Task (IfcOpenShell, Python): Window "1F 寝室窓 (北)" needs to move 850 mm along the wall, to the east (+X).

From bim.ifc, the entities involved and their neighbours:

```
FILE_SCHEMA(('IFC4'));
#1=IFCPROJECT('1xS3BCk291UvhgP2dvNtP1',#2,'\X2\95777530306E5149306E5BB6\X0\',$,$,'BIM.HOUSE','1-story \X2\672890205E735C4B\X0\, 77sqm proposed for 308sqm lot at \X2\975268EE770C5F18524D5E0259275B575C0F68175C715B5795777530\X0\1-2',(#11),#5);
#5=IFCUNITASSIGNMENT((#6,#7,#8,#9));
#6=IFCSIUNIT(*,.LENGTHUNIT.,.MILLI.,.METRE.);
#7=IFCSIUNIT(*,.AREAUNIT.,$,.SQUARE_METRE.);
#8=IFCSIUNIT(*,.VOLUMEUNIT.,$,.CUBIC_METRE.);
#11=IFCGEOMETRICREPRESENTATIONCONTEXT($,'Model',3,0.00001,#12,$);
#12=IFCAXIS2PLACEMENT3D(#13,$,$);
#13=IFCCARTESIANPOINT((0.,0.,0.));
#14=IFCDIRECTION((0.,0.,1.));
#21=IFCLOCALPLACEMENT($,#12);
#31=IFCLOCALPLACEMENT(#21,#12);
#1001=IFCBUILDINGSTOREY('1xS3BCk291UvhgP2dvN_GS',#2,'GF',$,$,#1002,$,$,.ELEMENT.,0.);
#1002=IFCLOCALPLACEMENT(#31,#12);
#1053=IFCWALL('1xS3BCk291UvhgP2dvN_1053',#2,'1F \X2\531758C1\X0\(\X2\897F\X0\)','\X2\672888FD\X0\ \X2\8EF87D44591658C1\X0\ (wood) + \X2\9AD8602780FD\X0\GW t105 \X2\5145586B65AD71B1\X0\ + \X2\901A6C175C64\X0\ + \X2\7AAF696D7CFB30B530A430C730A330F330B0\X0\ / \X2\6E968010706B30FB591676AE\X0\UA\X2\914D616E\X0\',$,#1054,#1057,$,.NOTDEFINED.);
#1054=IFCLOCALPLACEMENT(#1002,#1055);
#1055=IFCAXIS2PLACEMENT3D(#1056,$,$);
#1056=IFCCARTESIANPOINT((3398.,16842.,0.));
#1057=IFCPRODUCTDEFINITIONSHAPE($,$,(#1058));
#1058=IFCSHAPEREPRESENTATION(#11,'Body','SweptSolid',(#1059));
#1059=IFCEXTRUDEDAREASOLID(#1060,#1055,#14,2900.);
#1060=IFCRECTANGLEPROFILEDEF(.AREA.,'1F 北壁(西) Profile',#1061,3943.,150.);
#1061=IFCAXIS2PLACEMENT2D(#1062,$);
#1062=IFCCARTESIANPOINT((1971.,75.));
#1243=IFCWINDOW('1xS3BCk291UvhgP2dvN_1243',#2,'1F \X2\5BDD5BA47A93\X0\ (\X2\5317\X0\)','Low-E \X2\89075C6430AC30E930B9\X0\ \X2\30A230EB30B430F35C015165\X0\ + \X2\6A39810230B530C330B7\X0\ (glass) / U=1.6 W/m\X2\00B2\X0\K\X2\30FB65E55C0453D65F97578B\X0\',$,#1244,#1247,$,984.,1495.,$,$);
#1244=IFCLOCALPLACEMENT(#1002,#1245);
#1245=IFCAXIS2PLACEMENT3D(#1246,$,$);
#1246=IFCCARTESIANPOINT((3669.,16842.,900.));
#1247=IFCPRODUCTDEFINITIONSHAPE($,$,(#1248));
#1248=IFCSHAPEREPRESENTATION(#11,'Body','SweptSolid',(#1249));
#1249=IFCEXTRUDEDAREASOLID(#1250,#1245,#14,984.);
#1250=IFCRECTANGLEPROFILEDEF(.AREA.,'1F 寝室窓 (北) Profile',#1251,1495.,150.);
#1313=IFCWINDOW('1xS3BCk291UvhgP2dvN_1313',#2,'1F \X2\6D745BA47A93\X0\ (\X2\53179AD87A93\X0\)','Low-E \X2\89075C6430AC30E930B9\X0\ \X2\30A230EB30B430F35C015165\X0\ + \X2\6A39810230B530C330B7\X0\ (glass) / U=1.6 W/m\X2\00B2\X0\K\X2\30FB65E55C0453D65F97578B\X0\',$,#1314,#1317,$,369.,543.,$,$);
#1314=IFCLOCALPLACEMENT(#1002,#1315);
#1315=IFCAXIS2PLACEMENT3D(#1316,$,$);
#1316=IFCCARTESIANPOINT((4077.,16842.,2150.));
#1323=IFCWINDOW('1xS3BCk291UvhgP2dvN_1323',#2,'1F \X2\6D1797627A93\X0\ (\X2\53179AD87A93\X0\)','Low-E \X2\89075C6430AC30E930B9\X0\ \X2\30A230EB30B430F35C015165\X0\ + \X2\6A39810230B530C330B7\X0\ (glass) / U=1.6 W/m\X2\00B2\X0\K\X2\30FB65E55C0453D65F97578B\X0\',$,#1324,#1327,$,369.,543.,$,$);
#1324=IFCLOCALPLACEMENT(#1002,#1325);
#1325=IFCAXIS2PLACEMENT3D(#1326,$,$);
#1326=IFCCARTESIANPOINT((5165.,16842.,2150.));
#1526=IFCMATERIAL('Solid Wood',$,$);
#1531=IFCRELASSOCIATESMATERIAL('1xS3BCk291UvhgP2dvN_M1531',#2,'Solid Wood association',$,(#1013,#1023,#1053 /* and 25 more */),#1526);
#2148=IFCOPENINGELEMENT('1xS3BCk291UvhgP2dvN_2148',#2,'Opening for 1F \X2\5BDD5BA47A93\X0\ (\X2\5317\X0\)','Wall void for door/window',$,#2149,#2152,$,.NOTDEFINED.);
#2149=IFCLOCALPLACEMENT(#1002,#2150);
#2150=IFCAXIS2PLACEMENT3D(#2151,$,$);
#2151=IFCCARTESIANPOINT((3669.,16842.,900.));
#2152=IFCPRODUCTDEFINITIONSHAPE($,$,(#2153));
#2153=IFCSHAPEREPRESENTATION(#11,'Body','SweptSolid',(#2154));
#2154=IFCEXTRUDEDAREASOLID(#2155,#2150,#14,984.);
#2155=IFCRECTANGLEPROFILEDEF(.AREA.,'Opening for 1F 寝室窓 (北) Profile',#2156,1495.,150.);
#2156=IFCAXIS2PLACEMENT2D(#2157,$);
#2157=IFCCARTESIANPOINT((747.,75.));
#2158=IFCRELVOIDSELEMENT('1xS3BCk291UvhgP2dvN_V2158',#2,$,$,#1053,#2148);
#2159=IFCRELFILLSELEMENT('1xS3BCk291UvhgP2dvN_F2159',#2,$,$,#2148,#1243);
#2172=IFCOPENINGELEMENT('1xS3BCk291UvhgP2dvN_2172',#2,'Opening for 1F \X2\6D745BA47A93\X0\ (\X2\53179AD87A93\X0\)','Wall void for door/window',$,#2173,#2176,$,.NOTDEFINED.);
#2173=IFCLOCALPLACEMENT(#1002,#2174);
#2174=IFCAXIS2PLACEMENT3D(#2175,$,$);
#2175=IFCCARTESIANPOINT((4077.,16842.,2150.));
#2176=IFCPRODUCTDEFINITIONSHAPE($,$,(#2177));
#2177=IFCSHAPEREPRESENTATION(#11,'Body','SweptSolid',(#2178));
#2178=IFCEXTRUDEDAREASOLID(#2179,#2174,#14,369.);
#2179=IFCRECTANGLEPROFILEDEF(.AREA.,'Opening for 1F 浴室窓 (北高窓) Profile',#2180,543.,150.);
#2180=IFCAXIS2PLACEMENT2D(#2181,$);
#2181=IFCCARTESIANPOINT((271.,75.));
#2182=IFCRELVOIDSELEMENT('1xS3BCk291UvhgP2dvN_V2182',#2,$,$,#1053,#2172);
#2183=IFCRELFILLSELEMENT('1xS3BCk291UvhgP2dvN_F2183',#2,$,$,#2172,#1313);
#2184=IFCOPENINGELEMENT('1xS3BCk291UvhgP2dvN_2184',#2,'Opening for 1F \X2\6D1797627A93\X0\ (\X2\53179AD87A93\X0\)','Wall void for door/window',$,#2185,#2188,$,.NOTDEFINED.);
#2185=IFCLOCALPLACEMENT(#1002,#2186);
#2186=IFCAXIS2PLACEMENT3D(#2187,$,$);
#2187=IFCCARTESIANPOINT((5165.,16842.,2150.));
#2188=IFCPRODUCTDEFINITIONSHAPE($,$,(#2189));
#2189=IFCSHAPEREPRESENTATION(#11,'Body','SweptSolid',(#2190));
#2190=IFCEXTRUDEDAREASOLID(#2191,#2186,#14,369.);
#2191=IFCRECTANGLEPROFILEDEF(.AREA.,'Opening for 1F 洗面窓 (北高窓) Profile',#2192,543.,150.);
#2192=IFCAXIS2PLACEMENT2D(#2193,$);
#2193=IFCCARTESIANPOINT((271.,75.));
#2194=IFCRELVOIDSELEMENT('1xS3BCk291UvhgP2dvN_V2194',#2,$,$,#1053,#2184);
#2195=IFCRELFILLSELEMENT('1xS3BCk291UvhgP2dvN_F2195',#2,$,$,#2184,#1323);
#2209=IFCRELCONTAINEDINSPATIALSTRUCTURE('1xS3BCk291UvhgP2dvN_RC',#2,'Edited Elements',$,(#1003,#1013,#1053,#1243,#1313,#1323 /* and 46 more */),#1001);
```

```python
import ifcopenshell
import ifcopenshell.api.geometry
import ifcopenshell.util.placement
import ifcopenshell.util.unit

model = ifcopenshell.open("bim.ifc")
unit_scale = ifcopenshell.util.unit.calculate_unit_scale(model)

window = model.by_guid("1xS3BCk291UvhgP2dvN_1243")
opening = window.FillsVoids[0].RelatingOpeningElement
wall = opening.VoidsElements[0].RelatingBuildingElement

wall_matrix = ifcopenshell.util.placement.get_local_placement(wall.ObjectPlacement)
shift = wall_matrix[:3, 0] * 0.85 / unit_scale
before = ifcopenshell.util.placement.get_local_placement(window.ObjectPlacement)[:3, 3].copy()

# The window is not placed relative to its opening, so move both.
for product in (opening, window):
    matrix = ifcopenshell.util.placement.get_local_placement(product.ObjectPlacement)
    matrix[:3, 3] += shift
    ifcopenshell.api.geometry.edit_object_placement(model, product=product, matrix=matrix, is_si=False)

after = ifcopenshell.util.placement.get_local_placement(window.ObjectPlacement)[:3, 3]
print("window moved by", (after - before).round(3) + 0.0)

model.write("bim_rev.ifc")
```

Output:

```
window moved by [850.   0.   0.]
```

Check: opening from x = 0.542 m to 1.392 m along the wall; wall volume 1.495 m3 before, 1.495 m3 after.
